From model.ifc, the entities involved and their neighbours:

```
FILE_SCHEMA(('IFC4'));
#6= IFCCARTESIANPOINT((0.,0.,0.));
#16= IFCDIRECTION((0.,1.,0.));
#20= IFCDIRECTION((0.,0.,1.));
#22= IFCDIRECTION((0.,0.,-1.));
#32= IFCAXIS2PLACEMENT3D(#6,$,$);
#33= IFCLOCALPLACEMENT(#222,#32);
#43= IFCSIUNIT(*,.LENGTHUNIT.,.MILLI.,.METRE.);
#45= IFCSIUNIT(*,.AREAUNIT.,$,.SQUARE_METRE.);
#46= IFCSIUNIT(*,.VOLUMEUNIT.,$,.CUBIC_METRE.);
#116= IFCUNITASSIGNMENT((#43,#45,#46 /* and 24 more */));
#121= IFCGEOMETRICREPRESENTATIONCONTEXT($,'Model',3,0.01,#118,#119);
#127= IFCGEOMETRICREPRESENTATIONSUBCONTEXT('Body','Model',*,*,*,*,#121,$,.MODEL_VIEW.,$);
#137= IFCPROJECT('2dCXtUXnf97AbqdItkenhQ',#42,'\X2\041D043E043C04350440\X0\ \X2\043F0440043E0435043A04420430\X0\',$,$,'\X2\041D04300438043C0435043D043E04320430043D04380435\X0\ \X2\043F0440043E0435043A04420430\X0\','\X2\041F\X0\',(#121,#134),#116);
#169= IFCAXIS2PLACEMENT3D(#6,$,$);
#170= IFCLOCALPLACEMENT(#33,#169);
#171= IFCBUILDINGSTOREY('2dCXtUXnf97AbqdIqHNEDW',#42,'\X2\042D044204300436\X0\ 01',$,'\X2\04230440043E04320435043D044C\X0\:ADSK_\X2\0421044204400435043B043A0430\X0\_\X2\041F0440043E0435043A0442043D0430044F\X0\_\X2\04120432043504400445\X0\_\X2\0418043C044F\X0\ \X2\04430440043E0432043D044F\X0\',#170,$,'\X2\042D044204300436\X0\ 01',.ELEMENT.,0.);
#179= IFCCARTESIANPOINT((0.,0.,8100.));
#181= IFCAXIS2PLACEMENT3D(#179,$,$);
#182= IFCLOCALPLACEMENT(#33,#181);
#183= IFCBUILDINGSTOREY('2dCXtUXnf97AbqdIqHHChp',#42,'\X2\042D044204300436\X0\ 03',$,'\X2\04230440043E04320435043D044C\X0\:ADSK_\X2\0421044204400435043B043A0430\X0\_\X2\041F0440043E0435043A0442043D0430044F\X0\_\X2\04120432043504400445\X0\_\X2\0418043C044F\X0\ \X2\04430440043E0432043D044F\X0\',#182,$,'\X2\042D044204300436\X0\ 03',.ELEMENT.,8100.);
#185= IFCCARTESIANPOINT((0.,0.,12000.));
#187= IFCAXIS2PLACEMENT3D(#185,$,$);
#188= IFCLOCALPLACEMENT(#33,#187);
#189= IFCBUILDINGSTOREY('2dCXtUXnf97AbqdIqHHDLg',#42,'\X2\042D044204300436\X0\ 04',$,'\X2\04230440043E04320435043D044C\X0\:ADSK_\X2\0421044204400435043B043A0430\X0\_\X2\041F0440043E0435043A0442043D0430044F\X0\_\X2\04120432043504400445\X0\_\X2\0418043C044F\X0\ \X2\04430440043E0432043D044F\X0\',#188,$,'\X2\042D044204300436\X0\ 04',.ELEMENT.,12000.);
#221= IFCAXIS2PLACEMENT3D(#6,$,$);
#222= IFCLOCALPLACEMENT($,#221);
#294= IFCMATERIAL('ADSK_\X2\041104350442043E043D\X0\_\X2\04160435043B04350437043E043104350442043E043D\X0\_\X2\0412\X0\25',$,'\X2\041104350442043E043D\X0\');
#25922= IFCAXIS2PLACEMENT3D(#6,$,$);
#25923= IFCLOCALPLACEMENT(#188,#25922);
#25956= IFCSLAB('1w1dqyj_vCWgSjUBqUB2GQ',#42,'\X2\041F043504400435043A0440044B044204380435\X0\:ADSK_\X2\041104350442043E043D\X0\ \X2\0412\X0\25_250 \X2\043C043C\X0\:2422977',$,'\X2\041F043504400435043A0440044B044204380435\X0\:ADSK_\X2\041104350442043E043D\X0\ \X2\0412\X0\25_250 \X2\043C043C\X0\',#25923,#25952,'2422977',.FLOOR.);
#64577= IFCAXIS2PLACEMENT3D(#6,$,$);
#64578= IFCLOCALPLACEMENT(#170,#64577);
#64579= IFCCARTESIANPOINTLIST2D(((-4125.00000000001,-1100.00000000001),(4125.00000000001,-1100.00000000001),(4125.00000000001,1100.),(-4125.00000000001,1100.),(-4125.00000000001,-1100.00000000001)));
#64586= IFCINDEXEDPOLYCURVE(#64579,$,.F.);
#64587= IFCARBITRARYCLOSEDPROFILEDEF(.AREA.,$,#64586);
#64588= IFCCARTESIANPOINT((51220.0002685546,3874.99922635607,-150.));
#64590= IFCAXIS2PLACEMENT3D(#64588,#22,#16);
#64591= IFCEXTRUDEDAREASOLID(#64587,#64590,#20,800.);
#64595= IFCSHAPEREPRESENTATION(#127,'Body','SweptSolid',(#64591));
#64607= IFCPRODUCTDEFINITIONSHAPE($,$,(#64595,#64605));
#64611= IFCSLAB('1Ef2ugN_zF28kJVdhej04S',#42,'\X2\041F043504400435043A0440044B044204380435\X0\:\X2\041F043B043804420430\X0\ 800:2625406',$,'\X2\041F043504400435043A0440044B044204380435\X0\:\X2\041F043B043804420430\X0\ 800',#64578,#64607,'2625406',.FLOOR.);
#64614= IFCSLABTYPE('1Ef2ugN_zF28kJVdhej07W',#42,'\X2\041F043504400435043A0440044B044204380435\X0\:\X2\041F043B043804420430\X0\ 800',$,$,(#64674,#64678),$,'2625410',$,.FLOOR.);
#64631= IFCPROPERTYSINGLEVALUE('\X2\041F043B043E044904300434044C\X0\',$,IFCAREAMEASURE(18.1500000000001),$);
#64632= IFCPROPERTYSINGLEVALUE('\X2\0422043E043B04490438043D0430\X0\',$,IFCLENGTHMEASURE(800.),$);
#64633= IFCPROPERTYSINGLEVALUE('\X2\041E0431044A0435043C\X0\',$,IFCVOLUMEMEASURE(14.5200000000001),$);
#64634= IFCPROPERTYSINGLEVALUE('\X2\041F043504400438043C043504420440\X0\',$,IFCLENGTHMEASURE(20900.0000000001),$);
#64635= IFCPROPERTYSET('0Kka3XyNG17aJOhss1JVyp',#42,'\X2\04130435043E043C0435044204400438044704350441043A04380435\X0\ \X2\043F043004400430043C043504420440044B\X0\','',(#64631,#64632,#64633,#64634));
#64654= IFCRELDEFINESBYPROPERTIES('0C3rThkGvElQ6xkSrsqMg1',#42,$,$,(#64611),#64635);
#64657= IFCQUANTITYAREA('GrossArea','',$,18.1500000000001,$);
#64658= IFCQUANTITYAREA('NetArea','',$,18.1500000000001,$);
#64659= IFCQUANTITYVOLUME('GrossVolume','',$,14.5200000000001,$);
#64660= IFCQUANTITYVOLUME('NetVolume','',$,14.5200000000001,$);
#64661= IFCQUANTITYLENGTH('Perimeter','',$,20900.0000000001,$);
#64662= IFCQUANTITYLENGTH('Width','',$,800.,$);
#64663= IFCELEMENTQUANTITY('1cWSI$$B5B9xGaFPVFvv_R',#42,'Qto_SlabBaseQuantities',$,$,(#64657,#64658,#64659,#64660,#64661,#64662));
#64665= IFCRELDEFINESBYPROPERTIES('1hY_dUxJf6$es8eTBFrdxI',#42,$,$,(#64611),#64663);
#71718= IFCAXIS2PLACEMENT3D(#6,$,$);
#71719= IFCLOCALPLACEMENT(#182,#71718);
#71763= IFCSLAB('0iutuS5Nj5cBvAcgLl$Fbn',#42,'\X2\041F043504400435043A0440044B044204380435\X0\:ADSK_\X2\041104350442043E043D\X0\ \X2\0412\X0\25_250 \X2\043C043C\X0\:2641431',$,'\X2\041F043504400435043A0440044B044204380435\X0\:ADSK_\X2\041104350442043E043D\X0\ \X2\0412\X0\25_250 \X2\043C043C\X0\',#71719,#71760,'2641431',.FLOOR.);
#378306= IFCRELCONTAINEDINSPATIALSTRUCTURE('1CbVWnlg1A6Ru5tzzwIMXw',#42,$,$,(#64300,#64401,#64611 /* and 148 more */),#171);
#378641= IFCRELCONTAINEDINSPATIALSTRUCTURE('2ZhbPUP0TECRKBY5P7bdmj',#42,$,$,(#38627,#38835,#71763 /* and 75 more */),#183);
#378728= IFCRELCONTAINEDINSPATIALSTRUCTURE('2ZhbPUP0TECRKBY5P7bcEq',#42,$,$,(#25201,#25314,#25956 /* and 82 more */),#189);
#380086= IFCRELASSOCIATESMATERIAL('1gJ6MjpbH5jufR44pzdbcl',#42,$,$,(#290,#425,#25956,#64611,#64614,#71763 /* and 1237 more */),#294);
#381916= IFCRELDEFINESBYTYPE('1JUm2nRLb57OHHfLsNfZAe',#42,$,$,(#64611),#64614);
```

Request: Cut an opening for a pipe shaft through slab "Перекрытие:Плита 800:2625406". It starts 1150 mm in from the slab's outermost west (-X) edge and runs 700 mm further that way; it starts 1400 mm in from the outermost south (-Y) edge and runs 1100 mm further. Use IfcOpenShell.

```python
import numpy as np
import ifcopenshell
import ifcopenshell.api.feature
import ifcopenshell.api.geometry
import ifcopenshell.api.pset
import ifcopenshell.api.root
import ifcopenshell.geom
import ifcopenshell.util.element
import ifcopenshell.util.placement
import ifcopenshell.util.representation
import ifcopenshell.util.shape
import ifcopenshell.util.unit

model = ifcopenshell.open("model.ifc")
unit_scale = ifcopenshell.util.unit.calculate_unit_scale(model)
area_scale = ifcopenshell.util.unit.calculate_unit_scale(model, "AREAUNIT")
volume_scale = ifcopenshell.util.unit.calculate_unit_scale(model, "VOLUMEUNIT")
settings = ifcopenshell.geom.settings()


def volume(element):
    """Net volume in cubic metres, openings subtracted."""
    shape = ifcopenshell.geom.create_shape(settings, element)
    return ifcopenshell.util.shape.get_volume(shape.geometry)


slab = model.by_id(64611)
before = volume(slab)

# Extent in the slab's own axes, in metres. The edges named are its -X and -Y sides.
slab_shape = ifcopenshell.geom.create_shape(settings, slab)
vertices = ifcopenshell.util.shape.get_vertices(slab_shape.geometry)
x_min, y_min, bottom = vertices.min(axis=0)
top = vertices[:, 2].max()

opening = ifcopenshell.api.root.create_entity(model, ifc_class="IfcOpeningElement", name="Pipe shaft opening", predefined_type="OPENING")
context = ifcopenshell.util.representation.get_context(model, "Model", "Body", "MODEL_VIEW")
width, depth = 0.7, 1.1
outline = [(0.0, 0.0), (width, 0.0), (width, depth), (0.0, depth), (0.0, 0.0)]
# Overshoot both faces by 50 mm so the cut is clean.
shape = ifcopenshell.api.geometry.add_slab_representation(
    model, context=context, depth=top - bottom + 0.1, polyline=outline
)
ifcopenshell.api.geometry.assign_representation(model, product=opening, representation=shape)

matrix = ifcopenshell.util.placement.get_local_placement(slab.ObjectPlacement)
matrix[:, 3] = matrix @ np.append(np.array([x_min + 1.15, y_min + 1.4, bottom - 0.05]) / unit_scale, 1.0)
ifcopenshell.api.geometry.edit_object_placement(model, product=opening, matrix=matrix, is_si=False)
ifcopenshell.api.feature.add_feature(model, feature=opening, element=slab)

after = volume(slab)

# Update the slab's stored quantities.
pset = model.by_id(ifcopenshell.util.element.get_pset(slab, "Геометрические параметры", should_inherit=False)["id"])
ifcopenshell.api.pset.edit_pset(model, pset=pset, properties={
    "Площадь": model.create_entity("IfcAreaMeasure", after / (top - bottom) / area_scale),
    "Объем": model.create_entity("IfcVolumeMeasure", after / volume_scale),
})
qto = model.by_id(ifcopenshell.util.element.get_pset(slab, "Qto_SlabBaseQuantities", should_inherit=False)["id"])
ifcopenshell.api.pset.edit_qto(model, qto=qto, properties={
    "NetArea": after / (top - bottom) / area_scale,
    "NetVolume": after / volume_scale,
})

print(f"slab volume {before:.3f} -> {after:.3f} m3")

model.write("model_edited.ifc")
```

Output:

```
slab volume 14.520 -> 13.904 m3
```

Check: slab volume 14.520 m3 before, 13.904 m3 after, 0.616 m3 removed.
